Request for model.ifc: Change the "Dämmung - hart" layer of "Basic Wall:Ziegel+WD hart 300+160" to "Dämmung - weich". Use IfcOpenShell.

First a look at what the model holds.

```python
import ifcopenshell
import ifcopenshell.util.element

model = ifcopenshell.open("model.ifc")
print(model.schema)
for layer_set in model.by_type("IfcMaterialLayerSet"):
    if layer_set.LayerSetName == "Basic Wall:Ziegel+WD hart 300+160":
        for layer in layer_set.MaterialLayers:
            print(layer.id(), layer.Material and layer.Material.Name, layer.LayerThickness, sep=" | ")
        print(len(ifcopenshell.util.element.get_elements_by_material(model, layer_set)), "elements and types use it")
print(sorted(m.Name for m in model.by_type("IfcMaterial") if m.Name)[:60])
```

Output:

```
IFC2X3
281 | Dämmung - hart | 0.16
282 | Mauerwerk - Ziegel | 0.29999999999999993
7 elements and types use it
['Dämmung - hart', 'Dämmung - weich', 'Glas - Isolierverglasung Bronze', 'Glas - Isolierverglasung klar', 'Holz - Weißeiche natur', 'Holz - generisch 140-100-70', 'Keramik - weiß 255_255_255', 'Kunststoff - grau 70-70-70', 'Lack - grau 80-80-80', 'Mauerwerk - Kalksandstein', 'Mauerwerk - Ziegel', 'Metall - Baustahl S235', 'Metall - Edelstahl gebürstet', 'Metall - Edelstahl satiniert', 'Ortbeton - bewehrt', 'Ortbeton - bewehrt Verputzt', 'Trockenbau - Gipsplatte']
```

```python
import ifcopenshell
import ifcopenshell.api.material

model = ifcopenshell.open("model.ifc")

layer_set = next(s for s in model.by_type("IfcMaterialLayerSet") if s.LayerSetName == "Basic Wall:Ziegel+WD hart 300+160")
layer = next(l for l in layer_set.MaterialLayers if l.Material and l.Material.Name == "Dämmung - hart")
material = next(m for m in model.by_type("IfcMaterial") if m.Name == "Dämmung - weich")

# Point this one layer at the other material; renaming the old one would change it everywhere.
ifcopenshell.api.material.edit_layer(model, layer=layer, attributes={}, material=material)

print([l.Material.Name if l.Material else None for l in layer_set.MaterialLayers])

model.write("model-out.ifc")
```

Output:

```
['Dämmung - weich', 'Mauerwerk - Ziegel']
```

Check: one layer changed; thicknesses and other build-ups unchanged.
